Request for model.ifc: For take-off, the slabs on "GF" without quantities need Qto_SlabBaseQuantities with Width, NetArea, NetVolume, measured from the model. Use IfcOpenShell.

First a look at what the model holds.

```python
import ifcopenshell
import ifcopenshell.util.element
import ifcopenshell.util.unit

model = ifcopenshell.open("model.ifc")
print(model.schema)
for unit_type in ("LENGTHUNIT", "AREAUNIT", "VOLUMEUNIT"):
    print(unit_type, ifcopenshell.util.unit.calculate_unit_scale(model, unit_type))
storey = next(s for s in model.by_type("IfcBuildingStorey") if s.Name == "GF")
slabs = [e for e in ifcopenshell.util.element.get_decomposition(storey) if e.is_a("IfcSlab")]
for e in sorted(slabs, key=lambda e: e.id()):
    print(e.id(), e.is_a(), e.Name, list(ifcopenshell.util.element.get_psets(e, qtos_only=True)), sep=" | ")
```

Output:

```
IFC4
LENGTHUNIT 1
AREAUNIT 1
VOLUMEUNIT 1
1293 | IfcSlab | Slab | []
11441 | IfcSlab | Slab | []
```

```python
import ifcopenshell
import ifcopenshell.api.pset
import ifcopenshell.geom
import ifcopenshell.util.element
import ifcopenshell.util.shape
import ifcopenshell.util.unit

model = ifcopenshell.open("model.ifc")
unit_scale = ifcopenshell.util.unit.calculate_unit_scale(model)
area_scale = ifcopenshell.util.unit.calculate_unit_scale(model, "AREAUNIT")
volume_scale = ifcopenshell.util.unit.calculate_unit_scale(model, "VOLUMEUNIT")
settings = ifcopenshell.geom.settings()

storey = next(s for s in model.by_type("IfcBuildingStorey") if s.Name == "GF")
slabs = [e for e in ifcopenshell.util.element.get_decomposition(storey) if e.is_a("IfcSlab")]

for e in sorted(slabs, key=lambda e: e.id()):
    if ifcopenshell.util.element.get_psets(e, qtos_only=True, should_inherit=False):
        continue
    # Geometry comes back in metres, in the element's own axes.
    shape = ifcopenshell.geom.create_shape(settings, e)
    values = {
        "Width": ifcopenshell.util.shape.get_z(shape.geometry) / unit_scale,
        "NetArea": ifcopenshell.util.shape.get_footprint_area(shape.geometry) / area_scale,
        "NetVolume": ifcopenshell.util.shape.get_volume(shape.geometry) / volume_scale,
    }
    qto = ifcopenshell.api.pset.add_qto(model, product=e, name="Qto_SlabBaseQuantities")
    ifcopenshell.api.pset.edit_qto(model, qto=qto, properties=values)
    print(e.id(), {k: round(v, 3) for k, v in values.items()})

model.write("model-out.ifc")
```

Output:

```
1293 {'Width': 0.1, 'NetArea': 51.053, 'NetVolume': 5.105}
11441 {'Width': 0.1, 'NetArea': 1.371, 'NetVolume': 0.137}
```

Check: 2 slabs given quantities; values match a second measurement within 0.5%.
